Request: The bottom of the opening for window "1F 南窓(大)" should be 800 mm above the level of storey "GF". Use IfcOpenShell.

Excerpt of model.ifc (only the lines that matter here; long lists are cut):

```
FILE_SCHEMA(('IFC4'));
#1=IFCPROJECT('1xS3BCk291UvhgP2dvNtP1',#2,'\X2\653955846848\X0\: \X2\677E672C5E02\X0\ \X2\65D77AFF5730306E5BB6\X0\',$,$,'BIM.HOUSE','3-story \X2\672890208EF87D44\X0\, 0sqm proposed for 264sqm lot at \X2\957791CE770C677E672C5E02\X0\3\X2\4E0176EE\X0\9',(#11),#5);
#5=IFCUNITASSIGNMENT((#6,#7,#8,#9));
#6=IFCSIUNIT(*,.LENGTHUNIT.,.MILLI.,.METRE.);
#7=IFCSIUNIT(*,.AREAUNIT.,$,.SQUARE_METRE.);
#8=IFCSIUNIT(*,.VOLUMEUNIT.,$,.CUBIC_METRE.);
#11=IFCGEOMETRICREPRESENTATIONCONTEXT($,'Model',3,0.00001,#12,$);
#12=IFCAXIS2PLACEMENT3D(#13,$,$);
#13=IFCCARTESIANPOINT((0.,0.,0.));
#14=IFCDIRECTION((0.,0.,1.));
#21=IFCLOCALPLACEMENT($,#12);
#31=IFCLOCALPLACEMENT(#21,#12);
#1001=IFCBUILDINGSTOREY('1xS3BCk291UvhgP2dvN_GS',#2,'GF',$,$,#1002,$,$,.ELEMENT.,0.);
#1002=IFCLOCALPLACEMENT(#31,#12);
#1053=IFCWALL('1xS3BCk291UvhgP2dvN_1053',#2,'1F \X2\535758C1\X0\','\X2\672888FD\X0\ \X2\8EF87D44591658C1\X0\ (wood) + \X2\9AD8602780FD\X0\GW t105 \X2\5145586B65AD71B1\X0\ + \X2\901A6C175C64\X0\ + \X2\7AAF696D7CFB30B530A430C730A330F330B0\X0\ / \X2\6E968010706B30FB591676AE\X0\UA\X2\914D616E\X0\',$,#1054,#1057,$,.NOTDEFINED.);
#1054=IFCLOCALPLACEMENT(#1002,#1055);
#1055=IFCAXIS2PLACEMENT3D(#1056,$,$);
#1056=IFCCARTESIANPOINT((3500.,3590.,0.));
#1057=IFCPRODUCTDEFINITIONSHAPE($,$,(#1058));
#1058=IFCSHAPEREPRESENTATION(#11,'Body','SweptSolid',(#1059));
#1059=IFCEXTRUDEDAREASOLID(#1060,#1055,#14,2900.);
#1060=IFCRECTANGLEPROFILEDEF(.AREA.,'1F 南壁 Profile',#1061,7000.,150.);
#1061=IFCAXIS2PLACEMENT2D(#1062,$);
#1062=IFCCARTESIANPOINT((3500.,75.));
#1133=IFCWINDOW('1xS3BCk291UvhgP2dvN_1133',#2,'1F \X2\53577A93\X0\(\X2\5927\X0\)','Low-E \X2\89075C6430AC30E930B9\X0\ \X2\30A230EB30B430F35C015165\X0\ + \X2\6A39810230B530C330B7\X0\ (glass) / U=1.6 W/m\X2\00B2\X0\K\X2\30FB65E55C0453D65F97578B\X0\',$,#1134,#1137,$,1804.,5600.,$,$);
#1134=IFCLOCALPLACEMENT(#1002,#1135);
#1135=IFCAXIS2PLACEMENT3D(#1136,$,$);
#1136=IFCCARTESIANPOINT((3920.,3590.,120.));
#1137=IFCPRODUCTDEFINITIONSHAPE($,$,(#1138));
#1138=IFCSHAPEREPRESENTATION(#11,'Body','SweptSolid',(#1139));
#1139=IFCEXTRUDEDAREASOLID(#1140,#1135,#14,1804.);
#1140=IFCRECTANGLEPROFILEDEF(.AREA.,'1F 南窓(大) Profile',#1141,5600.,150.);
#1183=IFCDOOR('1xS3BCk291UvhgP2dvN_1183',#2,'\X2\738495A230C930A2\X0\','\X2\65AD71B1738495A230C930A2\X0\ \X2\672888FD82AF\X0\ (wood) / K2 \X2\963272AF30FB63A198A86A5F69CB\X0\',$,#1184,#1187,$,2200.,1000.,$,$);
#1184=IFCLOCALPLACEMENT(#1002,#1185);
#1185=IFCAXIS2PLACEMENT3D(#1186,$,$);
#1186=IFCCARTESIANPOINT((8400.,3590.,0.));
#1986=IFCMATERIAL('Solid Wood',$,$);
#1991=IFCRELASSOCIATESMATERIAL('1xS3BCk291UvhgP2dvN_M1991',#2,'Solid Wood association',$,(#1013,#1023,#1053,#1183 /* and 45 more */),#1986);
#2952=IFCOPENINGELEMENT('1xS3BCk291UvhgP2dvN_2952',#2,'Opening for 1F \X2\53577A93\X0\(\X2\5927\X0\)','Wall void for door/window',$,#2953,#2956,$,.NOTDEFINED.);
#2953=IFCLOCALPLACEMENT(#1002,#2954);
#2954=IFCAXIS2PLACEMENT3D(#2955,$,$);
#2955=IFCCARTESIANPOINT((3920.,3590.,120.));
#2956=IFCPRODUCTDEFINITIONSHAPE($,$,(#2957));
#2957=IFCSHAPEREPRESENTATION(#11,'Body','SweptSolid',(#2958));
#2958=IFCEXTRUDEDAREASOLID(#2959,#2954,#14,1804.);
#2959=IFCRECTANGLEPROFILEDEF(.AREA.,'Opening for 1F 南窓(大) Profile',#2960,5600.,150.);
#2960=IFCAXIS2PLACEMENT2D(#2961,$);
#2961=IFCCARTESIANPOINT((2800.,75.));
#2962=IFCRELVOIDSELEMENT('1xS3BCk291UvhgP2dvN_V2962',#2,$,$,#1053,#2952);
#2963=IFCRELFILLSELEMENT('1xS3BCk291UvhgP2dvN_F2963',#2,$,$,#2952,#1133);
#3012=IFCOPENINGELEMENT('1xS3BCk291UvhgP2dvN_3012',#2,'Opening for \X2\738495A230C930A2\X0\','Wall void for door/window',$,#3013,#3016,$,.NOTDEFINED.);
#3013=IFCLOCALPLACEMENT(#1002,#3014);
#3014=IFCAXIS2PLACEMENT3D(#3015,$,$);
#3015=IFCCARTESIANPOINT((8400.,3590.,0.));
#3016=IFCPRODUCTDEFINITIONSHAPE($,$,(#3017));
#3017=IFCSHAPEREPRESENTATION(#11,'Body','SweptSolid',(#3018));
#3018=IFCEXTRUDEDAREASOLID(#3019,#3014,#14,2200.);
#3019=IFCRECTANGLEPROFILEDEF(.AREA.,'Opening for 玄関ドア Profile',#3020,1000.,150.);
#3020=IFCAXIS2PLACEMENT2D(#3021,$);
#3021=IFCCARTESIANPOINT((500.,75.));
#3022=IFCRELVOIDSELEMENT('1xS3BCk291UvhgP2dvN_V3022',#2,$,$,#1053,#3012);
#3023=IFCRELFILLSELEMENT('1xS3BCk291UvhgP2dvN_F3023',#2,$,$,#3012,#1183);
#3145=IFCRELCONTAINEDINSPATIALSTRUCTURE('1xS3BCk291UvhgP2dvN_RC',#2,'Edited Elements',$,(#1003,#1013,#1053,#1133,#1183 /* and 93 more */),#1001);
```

```python
import numpy as np
import ifcopenshell
import ifcopenshell.api.geometry
import ifcopenshell.geom
import ifcopenshell.util.element
import ifcopenshell.util.placement
import ifcopenshell.util.shape
import ifcopenshell.util.unit

model = ifcopenshell.open("model.ifc")
unit_scale = ifcopenshell.util.unit.calculate_unit_scale(model)

window = model.by_guid("1xS3BCk291UvhgP2dvN_1133")
opening = window.FillsVoids[0].RelatingOpeningElement
storey = ifcopenshell.util.element.get_container(window, ifc_class="IfcBuildingStorey")
level = ifcopenshell.util.placement.get_local_placement(storey.ObjectPlacement)[2, 3]

# The opening's origin need not be at the sill, so measure its lowest point.
shape = ifcopenshell.geom.create_shape(ifcopenshell.geom.settings(), opening)
bottom = ifcopenshell.util.shape.get_shape_bottom_elevation(shape, shape.geometry) / unit_scale
dz = level + 0.8 / unit_scale - bottom

shift = np.array([0.0, 0.0, dz])
# The window is not placed relative to its opening, so move both.
for product in (opening, window):
    matrix = ifcopenshell.util.placement.get_local_placement(product.ObjectPlacement)
    matrix[:3, 3] += shift
    ifcopenshell.api.geometry.edit_object_placement(model, product=product, matrix=matrix, is_si=False)

print(f"moved by {dz * unit_scale:+.3f} m")

model.write("model_edited.ifc")
```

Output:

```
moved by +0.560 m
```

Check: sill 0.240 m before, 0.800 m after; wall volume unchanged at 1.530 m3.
